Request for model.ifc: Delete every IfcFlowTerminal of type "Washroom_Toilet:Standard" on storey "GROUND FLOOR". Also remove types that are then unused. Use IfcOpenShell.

First a look at what the model holds.

```python
import ifcopenshell
import ifcopenshell.util.element

model = ifcopenshell.open("model.ifc")
print(model.schema)
storey = next(s for s in model.by_type("IfcBuildingStorey") if s.Name == "GROUND FLOOR")
terminals = [e for e in ifcopenshell.util.element.get_decomposition(storey) if e.is_a("IfcFlowTerminal")]
seen = {}
for e in terminals:
    element_type = ifcopenshell.util.element.get_type(e)
    name = element_type.Name if element_type not in (None, e) else None
    seen[name] = seen.get(name, 0) + 1
for name, count in sorted(seen.items(), key=str):
    print(count, "x", name)
```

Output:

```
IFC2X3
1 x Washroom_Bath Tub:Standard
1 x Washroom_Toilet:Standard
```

```python
import ifcopenshell
import ifcopenshell.api.root
import ifcopenshell.util.element

model = ifcopenshell.open("model.ifc")

storey = next(s for s in model.by_type("IfcBuildingStorey") if s.Name == "GROUND FLOOR")
terminals = [e for e in ifcopenshell.util.element.get_decomposition(storey) if e.is_a("IfcFlowTerminal")]
targets = [e for e in terminals if (t := ifcopenshell.util.element.get_type(e)) not in (None, e) and t.Name == "Washroom_Toilet:Standard"]
types = {ifcopenshell.util.element.get_type(e) for e in targets} - {None, *targets}

for e in targets:
    ifcopenshell.api.root.remove_product(model, product=e)
print(len(targets), "removed")

unused = [t for t in types if not ifcopenshell.util.element.get_types(t)]
for t in unused:
    ifcopenshell.api.root.remove_product(model, product=t)
print(len(unused), "unused types removed")

model.write("model_rev.ifc")
```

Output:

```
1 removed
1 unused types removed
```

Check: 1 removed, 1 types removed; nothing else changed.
